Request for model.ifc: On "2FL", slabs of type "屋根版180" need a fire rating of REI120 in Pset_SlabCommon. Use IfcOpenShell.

First a look at what the model holds.

```python
import ifcopenshell
import ifcopenshell.util.element

model = ifcopenshell.open("model.ifc")
print(model.schema)
storey = next(s for s in model.by_type("IfcBuildingStorey") if s.Name == "2FL")
slabs = [e for e in ifcopenshell.util.element.get_decomposition(storey) if e.is_a("IfcSlab")]
seen = {}
for e in slabs:
    element_type = ifcopenshell.util.element.get_type(e)
    key = (element_type.Name if element_type != e and element_type else None, ifcopenshell.util.element.get_pset(e, "Pset_SlabCommon", "FireRating"))
    seen[key] = seen.get(key, 0) + 1
for (name, value), count in sorted(seen.items(), key=str):
    print(count, "x", name, "|", value)
```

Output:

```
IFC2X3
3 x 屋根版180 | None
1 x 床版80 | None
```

```python
import ifcopenshell
import ifcopenshell.api.pset
import ifcopenshell.util.element

model = ifcopenshell.open("model.ifc")

storey = next(s for s in model.by_type("IfcBuildingStorey") if s.Name == "2FL")
slabs = [e for e in ifcopenshell.util.element.get_decomposition(storey) if e.is_a("IfcSlab")]

count = 0
for e in slabs:
    element_type = ifcopenshell.util.element.get_type(e)
    if element_type in (None, e) or element_type.Name != "屋根版180":
        continue
    # add_pset returns the element's existing set when there is one.
    pset = ifcopenshell.api.pset.add_pset(model, product=e, name="Pset_SlabCommon")
    ifcopenshell.api.pset.edit_pset(model, pset=pset, properties={"FireRating": "REI120"})
    count += 1

print(count, "slabs updated")

model.write("model_rev.ifc")
```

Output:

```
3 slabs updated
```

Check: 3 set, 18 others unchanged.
